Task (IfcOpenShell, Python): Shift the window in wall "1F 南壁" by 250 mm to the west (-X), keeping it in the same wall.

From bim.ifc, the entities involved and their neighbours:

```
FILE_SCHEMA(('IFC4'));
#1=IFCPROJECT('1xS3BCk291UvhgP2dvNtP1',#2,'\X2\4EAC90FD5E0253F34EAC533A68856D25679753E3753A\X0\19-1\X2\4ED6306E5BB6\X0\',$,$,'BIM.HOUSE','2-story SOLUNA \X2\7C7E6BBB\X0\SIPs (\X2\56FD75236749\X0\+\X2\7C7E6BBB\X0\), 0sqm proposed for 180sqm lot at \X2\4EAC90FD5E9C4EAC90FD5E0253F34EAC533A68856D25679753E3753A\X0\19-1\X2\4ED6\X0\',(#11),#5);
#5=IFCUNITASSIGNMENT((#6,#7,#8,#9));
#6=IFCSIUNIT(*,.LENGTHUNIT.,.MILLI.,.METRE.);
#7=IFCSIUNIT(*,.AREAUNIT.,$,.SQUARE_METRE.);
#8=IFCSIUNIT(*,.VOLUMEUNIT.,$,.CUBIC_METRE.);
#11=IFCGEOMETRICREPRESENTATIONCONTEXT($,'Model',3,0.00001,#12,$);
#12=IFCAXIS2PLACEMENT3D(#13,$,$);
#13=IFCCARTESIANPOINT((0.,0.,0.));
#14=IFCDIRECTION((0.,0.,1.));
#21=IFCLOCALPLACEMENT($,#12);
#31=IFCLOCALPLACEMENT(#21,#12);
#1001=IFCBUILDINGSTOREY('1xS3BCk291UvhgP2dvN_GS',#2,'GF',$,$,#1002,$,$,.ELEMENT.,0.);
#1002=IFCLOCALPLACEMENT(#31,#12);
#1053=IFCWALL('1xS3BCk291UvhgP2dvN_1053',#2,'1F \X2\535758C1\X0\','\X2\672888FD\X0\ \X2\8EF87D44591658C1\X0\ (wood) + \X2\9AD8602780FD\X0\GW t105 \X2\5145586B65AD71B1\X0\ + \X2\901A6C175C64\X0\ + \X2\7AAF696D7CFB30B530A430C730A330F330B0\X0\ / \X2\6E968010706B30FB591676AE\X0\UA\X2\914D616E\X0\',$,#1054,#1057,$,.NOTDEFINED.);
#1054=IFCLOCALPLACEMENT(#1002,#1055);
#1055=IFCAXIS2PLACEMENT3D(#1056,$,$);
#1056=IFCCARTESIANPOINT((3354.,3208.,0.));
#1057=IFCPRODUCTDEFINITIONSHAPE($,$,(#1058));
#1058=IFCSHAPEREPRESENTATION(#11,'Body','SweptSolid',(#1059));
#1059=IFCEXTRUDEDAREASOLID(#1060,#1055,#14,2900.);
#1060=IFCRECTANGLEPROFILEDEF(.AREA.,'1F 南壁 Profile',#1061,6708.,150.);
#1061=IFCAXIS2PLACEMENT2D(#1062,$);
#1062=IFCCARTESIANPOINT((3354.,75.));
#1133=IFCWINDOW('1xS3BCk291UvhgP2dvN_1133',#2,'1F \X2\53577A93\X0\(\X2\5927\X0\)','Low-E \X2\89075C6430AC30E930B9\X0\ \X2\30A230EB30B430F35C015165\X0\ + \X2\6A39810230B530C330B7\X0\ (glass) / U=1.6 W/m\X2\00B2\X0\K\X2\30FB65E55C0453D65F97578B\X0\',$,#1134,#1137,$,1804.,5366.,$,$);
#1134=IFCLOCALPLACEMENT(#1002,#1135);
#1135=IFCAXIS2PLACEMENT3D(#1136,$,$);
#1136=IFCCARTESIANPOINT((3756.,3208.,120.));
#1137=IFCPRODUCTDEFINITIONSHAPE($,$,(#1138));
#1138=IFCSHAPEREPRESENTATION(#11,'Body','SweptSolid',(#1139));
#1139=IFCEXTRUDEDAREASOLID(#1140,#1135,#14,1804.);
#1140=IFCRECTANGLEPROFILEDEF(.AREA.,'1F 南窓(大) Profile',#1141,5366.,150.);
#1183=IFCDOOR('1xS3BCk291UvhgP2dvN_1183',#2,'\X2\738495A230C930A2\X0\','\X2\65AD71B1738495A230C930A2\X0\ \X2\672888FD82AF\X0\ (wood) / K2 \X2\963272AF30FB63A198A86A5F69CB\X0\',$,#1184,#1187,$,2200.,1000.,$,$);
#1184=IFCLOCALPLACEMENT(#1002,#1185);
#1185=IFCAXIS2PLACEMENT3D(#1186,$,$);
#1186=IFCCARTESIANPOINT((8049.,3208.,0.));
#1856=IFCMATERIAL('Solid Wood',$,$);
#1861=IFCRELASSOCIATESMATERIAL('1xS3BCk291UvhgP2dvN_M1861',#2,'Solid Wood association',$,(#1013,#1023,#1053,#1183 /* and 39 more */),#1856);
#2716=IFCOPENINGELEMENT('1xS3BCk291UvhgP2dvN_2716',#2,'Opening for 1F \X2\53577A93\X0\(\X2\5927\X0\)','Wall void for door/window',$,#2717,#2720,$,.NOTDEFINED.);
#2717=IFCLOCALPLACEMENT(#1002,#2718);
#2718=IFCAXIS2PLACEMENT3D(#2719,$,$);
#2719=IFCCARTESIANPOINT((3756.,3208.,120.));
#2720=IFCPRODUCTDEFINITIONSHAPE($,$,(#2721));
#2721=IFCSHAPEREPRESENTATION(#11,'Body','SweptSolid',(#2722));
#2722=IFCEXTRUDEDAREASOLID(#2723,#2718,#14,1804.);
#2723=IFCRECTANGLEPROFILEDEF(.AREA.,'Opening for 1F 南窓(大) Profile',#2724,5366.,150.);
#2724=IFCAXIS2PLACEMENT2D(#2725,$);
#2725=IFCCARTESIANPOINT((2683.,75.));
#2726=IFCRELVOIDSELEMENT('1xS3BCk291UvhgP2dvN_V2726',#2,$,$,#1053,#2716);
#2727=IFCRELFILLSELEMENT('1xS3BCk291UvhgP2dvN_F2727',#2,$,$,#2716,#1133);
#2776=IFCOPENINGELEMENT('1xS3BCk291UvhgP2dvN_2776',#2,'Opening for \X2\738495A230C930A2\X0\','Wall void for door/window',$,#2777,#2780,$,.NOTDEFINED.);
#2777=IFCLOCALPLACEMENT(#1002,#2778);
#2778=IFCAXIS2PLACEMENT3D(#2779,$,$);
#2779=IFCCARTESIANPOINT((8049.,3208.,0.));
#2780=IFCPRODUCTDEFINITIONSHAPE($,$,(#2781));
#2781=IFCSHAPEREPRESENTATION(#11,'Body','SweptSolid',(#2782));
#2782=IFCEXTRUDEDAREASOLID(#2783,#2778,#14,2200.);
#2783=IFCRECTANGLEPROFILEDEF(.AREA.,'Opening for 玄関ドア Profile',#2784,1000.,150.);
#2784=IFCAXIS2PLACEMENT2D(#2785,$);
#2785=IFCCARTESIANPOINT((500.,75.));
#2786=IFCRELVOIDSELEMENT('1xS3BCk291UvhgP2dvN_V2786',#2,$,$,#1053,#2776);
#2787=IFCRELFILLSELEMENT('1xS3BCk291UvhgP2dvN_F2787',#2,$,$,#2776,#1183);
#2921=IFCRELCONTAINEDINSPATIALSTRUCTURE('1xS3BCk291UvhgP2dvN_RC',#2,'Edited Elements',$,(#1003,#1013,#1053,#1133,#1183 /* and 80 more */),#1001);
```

```python
import ifcopenshell
import ifcopenshell.api.geometry
import ifcopenshell.util.placement
import ifcopenshell.util.unit

model = ifcopenshell.open("bim.ifc")
unit_scale = ifcopenshell.util.unit.calculate_unit_scale(model)

window = model.by_guid("1xS3BCk291UvhgP2dvN_1133")
opening = window.FillsVoids[0].RelatingOpeningElement
wall = opening.VoidsElements[0].RelatingBuildingElement

wall_matrix = ifcopenshell.util.placement.get_local_placement(wall.ObjectPlacement)
shift = wall_matrix[:3, 0] * -0.25 / unit_scale
before = ifcopenshell.util.placement.get_local_placement(window.ObjectPlacement)[:3, 3].copy()

# The window is not placed relative to its opening, so move both.
for product in (opening, window):
    matrix = ifcopenshell.util.placement.get_local_placement(product.ObjectPlacement)
    matrix[:3, 3] += shift
    ifcopenshell.api.geometry.edit_object_placement(model, product=product, matrix=matrix, is_si=False)

after = ifcopenshell.util.placement.get_local_placement(window.ObjectPlacement)[:3, 3]
print("window moved by", (after - before).round(3) + 0.0)

model.write("bim_updated.ifc")
```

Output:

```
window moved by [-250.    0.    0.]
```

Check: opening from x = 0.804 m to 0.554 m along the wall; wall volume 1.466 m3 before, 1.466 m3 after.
